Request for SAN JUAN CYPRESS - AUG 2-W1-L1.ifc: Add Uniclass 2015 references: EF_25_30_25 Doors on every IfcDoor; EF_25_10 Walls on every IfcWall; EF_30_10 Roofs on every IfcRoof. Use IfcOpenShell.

First a look at what the model holds.

```python
import ifcopenshell

model = ifcopenshell.open("SAN JUAN CYPRESS - AUG 2-W1-L1.ifc")
print(model.schema)
print("classifications:", [c.Name for c in model.by_type("IfcClassification")])
for ifc_class in ("IfcDoor", "IfcRoof", "IfcStair", "IfcWall", "IfcWindow"):
    print(ifc_class, len(model.by_type(ifc_class)))
```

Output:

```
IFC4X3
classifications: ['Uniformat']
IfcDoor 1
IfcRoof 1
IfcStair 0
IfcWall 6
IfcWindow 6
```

```python
import ifcopenshell
import ifcopenshell.api.classification

model = ifcopenshell.open("SAN JUAN CYPRESS - AUG 2-W1-L1.ifc")

system = ifcopenshell.api.classification.add_classification(model, classification="Uniclass 2015")

codes = {
    "IfcDoor": ("EF_25_30_25", "Doors"),
    "IfcWall": ("EF_25_10", "Walls"),
    "IfcRoof": ("EF_30_10", "Roofs"),
}
for ifc_class, (code, name) in codes.items():
    products = model.by_type(ifc_class)
    ifcopenshell.api.classification.add_reference(
        model, products=products, classification=system, identification=code, name=name
    )
    print(code, len(products))

model.write("SAN JUAN CYPRESS - AUG 2-W1-L1_updated.ifc")
```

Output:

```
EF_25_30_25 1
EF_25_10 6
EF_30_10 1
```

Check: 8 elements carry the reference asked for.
